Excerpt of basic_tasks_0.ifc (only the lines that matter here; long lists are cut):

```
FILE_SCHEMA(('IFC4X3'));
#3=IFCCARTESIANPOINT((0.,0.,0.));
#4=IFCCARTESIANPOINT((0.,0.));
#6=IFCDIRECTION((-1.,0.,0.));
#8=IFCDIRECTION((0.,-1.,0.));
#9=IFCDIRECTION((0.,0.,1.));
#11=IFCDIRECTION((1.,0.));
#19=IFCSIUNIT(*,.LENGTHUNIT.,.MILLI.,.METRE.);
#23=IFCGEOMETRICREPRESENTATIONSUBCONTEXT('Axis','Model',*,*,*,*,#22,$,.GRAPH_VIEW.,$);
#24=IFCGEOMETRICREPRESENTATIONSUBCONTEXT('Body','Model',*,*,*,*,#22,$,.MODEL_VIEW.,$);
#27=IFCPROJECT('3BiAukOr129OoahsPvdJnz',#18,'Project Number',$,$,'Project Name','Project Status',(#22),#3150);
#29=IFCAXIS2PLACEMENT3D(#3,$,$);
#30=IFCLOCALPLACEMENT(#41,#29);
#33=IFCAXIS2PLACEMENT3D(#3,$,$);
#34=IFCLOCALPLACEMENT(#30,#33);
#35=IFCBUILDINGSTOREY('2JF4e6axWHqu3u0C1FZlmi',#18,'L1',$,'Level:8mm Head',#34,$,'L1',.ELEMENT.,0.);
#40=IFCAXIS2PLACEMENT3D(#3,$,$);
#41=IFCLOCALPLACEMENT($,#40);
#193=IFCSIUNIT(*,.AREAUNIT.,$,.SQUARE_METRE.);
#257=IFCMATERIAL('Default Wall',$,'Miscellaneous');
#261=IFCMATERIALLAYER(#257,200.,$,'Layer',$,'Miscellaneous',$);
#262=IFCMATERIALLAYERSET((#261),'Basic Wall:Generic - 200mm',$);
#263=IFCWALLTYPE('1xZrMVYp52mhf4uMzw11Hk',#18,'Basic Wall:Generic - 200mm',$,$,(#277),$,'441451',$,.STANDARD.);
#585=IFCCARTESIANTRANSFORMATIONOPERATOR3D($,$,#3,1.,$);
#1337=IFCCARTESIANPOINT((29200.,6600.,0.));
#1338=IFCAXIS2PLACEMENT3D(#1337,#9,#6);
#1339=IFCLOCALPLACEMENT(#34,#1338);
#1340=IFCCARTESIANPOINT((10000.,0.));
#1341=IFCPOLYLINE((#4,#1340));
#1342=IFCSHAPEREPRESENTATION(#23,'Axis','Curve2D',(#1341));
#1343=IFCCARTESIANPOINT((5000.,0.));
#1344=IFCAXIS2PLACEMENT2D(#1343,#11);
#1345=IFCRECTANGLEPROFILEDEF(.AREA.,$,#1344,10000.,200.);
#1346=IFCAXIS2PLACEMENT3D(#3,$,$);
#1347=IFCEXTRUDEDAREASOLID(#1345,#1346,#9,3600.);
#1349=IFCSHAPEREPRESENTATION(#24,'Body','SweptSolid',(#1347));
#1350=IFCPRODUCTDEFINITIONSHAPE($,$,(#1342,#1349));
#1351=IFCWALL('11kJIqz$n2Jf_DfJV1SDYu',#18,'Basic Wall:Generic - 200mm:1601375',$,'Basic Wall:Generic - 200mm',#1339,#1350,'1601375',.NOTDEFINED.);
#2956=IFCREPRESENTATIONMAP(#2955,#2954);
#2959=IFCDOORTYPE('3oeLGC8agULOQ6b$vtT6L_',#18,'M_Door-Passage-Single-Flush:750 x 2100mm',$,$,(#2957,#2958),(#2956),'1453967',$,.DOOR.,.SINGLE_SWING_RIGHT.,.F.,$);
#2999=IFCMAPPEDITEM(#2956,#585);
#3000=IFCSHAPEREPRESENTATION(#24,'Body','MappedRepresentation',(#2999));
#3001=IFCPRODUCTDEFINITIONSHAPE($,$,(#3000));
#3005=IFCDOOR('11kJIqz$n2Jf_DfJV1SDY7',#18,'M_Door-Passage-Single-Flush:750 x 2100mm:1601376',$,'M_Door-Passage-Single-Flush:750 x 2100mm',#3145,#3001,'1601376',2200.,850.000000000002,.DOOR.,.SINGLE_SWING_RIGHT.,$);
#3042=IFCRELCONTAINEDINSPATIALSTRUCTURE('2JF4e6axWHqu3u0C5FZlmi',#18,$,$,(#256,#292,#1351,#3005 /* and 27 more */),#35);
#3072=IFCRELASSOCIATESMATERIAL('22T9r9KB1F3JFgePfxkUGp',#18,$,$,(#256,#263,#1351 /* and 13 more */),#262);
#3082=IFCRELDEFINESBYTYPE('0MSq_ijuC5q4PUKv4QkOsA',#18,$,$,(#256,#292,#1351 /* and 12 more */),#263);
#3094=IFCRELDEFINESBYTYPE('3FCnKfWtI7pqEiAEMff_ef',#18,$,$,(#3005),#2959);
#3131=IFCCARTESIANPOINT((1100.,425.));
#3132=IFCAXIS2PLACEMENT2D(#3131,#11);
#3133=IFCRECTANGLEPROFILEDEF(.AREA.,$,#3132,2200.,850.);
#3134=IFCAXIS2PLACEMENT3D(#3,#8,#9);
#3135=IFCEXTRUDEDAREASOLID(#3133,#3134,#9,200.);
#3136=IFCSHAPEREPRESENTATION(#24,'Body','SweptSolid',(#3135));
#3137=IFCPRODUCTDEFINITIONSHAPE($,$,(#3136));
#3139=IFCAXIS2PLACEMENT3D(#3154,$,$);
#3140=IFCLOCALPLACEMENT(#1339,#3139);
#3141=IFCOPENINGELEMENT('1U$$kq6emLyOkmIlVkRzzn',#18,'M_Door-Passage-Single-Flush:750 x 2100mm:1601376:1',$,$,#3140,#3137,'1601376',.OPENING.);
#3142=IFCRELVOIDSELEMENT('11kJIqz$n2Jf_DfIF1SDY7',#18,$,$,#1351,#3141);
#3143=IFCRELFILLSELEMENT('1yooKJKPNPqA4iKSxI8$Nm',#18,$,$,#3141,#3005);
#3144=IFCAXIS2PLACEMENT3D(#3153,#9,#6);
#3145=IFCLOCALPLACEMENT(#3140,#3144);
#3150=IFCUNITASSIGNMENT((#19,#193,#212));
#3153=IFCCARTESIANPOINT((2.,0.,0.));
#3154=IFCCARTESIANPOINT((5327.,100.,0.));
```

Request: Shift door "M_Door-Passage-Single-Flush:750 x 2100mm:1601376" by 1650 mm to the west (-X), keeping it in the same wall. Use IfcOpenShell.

```python
import ifcopenshell
import ifcopenshell.api.geometry
import ifcopenshell.util.placement
import ifcopenshell.util.unit

model = ifcopenshell.open("basic_tasks_0.ifc")
unit_scale = ifcopenshell.util.unit.calculate_unit_scale(model)

door = model.by_guid("11kJIqz$n2Jf_DfJV1SDY7")
opening = door.FillsVoids[0].RelatingOpeningElement
wall = opening.VoidsElements[0].RelatingBuildingElement

wall_matrix = ifcopenshell.util.placement.get_local_placement(wall.ObjectPlacement)
shift = wall_matrix[:3, 0] * 1.65 / unit_scale
before = ifcopenshell.util.placement.get_local_placement(door.ObjectPlacement)[:3, 3].copy()

# The door is placed relative to its opening, so it follows when the opening moves.
matrix = ifcopenshell.util.placement.get_local_placement(opening.ObjectPlacement)
matrix[:3, 3] += shift
ifcopenshell.api.geometry.edit_object_placement(
    model, product=opening, matrix=matrix, is_si=False, should_transform_children=True
)

after = ifcopenshell.util.placement.get_local_placement(door.ObjectPlacement)[:3, 3]
print("door moved by", (after - before).round(3) + 0.0)

model.write("basic_tasks_0_rev.ifc")
```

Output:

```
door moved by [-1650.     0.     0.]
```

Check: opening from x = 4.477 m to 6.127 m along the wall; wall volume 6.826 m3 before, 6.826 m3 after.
